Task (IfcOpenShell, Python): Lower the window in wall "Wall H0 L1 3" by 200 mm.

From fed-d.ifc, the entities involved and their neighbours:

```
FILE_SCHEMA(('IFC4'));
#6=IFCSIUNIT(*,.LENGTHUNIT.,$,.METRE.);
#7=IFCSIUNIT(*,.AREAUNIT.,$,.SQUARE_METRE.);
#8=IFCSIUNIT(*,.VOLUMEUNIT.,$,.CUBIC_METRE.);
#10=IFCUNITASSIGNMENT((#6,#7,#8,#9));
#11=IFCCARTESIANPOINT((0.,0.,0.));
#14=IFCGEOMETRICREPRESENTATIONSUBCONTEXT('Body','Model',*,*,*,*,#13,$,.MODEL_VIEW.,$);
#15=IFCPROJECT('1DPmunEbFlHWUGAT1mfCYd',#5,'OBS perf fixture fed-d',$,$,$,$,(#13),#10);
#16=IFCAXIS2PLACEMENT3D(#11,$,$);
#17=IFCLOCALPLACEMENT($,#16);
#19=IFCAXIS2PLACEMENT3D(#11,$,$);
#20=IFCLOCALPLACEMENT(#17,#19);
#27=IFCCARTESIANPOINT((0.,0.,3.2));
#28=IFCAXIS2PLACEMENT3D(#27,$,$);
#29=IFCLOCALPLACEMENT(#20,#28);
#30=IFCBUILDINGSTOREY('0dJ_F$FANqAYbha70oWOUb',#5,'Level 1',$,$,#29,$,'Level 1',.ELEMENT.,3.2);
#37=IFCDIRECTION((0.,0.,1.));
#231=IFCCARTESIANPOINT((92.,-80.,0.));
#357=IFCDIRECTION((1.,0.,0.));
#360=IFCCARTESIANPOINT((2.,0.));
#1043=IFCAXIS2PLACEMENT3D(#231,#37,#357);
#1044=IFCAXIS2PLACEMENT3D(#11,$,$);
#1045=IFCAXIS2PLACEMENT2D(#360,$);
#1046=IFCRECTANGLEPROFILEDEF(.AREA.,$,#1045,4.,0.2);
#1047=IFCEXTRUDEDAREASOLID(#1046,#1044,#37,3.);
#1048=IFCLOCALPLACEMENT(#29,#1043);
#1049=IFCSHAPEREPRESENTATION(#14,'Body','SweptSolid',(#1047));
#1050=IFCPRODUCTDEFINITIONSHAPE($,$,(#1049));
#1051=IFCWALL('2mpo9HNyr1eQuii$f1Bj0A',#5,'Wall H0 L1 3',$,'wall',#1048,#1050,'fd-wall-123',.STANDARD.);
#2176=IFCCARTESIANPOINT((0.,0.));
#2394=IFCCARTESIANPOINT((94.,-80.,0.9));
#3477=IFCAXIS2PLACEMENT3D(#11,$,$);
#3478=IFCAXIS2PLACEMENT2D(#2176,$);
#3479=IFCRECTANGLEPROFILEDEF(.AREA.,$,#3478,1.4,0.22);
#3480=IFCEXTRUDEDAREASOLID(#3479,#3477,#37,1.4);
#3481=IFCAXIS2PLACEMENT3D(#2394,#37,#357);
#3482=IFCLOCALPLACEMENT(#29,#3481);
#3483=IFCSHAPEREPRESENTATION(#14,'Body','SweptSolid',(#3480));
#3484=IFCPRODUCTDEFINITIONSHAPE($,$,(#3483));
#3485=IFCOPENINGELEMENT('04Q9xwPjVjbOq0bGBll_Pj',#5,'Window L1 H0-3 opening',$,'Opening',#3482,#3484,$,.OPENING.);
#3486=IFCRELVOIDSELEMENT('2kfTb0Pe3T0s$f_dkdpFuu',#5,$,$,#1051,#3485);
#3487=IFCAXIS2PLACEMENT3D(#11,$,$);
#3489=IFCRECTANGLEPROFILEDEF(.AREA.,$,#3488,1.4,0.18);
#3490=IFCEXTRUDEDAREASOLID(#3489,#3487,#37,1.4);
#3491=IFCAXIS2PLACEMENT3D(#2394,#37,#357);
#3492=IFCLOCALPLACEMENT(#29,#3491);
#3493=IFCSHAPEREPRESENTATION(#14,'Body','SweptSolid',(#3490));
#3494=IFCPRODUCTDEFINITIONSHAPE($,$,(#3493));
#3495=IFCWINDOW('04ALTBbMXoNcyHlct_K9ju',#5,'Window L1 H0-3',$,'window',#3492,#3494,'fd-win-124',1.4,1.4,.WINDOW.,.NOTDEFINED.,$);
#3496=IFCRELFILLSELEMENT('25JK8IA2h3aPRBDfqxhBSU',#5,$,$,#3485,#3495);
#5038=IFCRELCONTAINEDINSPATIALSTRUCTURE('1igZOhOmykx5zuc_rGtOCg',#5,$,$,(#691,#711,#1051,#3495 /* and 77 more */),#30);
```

```python
import numpy as np
import ifcopenshell
import ifcopenshell.api.geometry
import ifcopenshell.util.placement
import ifcopenshell.util.unit

model = ifcopenshell.open("fed-d.ifc")
unit_scale = ifcopenshell.util.unit.calculate_unit_scale(model)

window = model.by_guid("04ALTBbMXoNcyHlct_K9ju")
opening = window.FillsVoids[0].RelatingOpeningElement
dz = -0.2

shift = np.array([0.0, 0.0, dz])
# The window is not placed relative to its opening, so move both.
for product in (opening, window):
    matrix = ifcopenshell.util.placement.get_local_placement(product.ObjectPlacement)
    matrix[:3, 3] += shift
    ifcopenshell.api.geometry.edit_object_placement(model, product=product, matrix=matrix, is_si=False)

print(f"moved by {dz * unit_scale:+.3f} m")

model.write("fed-d_edited.ifc")
```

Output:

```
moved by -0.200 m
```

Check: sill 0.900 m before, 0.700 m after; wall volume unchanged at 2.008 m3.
